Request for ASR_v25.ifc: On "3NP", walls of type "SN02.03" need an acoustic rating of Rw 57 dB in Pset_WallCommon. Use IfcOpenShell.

First a look at what the model holds.

```python
import ifcopenshell
import ifcopenshell.util.element

model = ifcopenshell.open("ASR_v25.ifc")
print(model.schema)
storey = next(s for s in model.by_type("IfcBuildingStorey") if s.Name == "3NP")
walls = [e for e in ifcopenshell.util.element.get_decomposition(storey) if e.is_a("IfcWall")]
seen = {}
for e in walls:
    element_type = ifcopenshell.util.element.get_type(e)
    key = (element_type.Name if element_type != e and element_type else None, ifcopenshell.util.element.get_pset(e, "Pset_WallCommon", "AcousticRating"))
    seen[key] = seen.get(key, 0) + 1
for (name, value), count in sorted(seen.items(), key=str):
    print(count, "x", name, "|", value)
```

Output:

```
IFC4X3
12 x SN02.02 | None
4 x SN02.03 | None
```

```python
import ifcopenshell
import ifcopenshell.api.pset
import ifcopenshell.util.element

model = ifcopenshell.open("ASR_v25.ifc")

storey = next(s for s in model.by_type("IfcBuildingStorey") if s.Name == "3NP")
walls = [e for e in ifcopenshell.util.element.get_decomposition(storey) if e.is_a("IfcWall")]

count = 0
for e in walls:
    element_type = ifcopenshell.util.element.get_type(e)
    if element_type in (None, e) or element_type.Name != "SN02.03":
        continue
    # add_pset returns the element's existing set when there is one.
    pset = ifcopenshell.api.pset.add_pset(model, product=e, name="Pset_WallCommon")
    ifcopenshell.api.pset.edit_pset(model, pset=pset, properties={"AcousticRating": "Rw 57 dB"})
    count += 1

print(count, "walls updated")

model.write("ASR_v25_edited.ifc")
```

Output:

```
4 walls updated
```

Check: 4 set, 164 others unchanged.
